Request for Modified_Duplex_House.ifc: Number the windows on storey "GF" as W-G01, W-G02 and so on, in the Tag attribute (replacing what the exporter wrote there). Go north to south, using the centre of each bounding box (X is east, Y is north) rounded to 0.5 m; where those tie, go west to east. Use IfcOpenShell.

First a look at what the model holds.

```python
import ifcopenshell
import ifcopenshell.util.element
import ifcopenshell.util.placement

model = ifcopenshell.open("Modified_Duplex_House.ifc")
print(model.schema)
storey = next(s for s in model.by_type("IfcBuildingStorey") if s.Name == "GF")
windows = [e for e in ifcopenshell.util.element.get_decomposition(storey) if e.is_a("IfcWindow")]
for e in sorted(windows, key=lambda e: e.id()):
    origin = ifcopenshell.util.placement.get_local_placement(e.ObjectPlacement)[:3, 3]
    print(e.id(), e.Tag, e.Name, origin.round(2) + 0.0, sep=" | ")
```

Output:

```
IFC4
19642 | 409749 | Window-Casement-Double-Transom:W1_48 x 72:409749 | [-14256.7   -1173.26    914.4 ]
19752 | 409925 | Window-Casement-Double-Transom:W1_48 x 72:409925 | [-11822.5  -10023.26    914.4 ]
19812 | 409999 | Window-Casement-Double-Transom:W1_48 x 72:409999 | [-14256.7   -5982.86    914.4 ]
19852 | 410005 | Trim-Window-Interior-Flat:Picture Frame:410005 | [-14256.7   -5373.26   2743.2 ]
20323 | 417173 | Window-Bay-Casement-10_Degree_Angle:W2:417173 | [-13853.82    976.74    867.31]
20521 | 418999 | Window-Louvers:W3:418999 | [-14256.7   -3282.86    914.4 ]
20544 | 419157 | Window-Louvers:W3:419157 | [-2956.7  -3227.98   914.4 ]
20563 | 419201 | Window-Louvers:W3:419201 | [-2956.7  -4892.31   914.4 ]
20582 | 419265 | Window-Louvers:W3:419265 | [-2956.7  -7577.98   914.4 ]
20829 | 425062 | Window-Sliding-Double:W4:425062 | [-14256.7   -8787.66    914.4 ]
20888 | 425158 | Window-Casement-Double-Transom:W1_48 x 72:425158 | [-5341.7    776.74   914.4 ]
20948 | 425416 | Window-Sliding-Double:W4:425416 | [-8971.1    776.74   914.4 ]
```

```python
import ifcopenshell
import ifcopenshell.geom
import ifcopenshell.util.element
import ifcopenshell.util.shape

model = ifcopenshell.open("Modified_Duplex_House.ifc")
settings = ifcopenshell.geom.settings()
settings.set("use-world-coords", True)


def centre(element):
    shape = ifcopenshell.geom.create_shape(settings, element)
    return ifcopenshell.util.shape.get_bbox_centroid(shape.geometry)


storey = next(s for s in model.by_type("IfcBuildingStorey") if s.Name == "GF")
windows = [e for e in ifcopenshell.util.element.get_decomposition(storey) if e.is_a("IfcWindow")]

# Insertion points can sit at a corner or the storey origin, so sort by the geometry (in metres).
centres = {e: centre(e) for e in windows}
windows.sort(key=lambda e: (-round(centres[e][1] / 0.5), centres[e][0]))

for i, e in enumerate(windows, start=1):
    number = f"W-G{i:02d}"
    e.Tag = number
    print(e.id(), number)

model.write("Modified_Duplex_House_v2.ifc")
```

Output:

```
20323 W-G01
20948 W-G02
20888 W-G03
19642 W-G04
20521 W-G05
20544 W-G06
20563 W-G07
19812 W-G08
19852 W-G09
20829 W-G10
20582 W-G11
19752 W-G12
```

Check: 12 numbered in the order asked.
